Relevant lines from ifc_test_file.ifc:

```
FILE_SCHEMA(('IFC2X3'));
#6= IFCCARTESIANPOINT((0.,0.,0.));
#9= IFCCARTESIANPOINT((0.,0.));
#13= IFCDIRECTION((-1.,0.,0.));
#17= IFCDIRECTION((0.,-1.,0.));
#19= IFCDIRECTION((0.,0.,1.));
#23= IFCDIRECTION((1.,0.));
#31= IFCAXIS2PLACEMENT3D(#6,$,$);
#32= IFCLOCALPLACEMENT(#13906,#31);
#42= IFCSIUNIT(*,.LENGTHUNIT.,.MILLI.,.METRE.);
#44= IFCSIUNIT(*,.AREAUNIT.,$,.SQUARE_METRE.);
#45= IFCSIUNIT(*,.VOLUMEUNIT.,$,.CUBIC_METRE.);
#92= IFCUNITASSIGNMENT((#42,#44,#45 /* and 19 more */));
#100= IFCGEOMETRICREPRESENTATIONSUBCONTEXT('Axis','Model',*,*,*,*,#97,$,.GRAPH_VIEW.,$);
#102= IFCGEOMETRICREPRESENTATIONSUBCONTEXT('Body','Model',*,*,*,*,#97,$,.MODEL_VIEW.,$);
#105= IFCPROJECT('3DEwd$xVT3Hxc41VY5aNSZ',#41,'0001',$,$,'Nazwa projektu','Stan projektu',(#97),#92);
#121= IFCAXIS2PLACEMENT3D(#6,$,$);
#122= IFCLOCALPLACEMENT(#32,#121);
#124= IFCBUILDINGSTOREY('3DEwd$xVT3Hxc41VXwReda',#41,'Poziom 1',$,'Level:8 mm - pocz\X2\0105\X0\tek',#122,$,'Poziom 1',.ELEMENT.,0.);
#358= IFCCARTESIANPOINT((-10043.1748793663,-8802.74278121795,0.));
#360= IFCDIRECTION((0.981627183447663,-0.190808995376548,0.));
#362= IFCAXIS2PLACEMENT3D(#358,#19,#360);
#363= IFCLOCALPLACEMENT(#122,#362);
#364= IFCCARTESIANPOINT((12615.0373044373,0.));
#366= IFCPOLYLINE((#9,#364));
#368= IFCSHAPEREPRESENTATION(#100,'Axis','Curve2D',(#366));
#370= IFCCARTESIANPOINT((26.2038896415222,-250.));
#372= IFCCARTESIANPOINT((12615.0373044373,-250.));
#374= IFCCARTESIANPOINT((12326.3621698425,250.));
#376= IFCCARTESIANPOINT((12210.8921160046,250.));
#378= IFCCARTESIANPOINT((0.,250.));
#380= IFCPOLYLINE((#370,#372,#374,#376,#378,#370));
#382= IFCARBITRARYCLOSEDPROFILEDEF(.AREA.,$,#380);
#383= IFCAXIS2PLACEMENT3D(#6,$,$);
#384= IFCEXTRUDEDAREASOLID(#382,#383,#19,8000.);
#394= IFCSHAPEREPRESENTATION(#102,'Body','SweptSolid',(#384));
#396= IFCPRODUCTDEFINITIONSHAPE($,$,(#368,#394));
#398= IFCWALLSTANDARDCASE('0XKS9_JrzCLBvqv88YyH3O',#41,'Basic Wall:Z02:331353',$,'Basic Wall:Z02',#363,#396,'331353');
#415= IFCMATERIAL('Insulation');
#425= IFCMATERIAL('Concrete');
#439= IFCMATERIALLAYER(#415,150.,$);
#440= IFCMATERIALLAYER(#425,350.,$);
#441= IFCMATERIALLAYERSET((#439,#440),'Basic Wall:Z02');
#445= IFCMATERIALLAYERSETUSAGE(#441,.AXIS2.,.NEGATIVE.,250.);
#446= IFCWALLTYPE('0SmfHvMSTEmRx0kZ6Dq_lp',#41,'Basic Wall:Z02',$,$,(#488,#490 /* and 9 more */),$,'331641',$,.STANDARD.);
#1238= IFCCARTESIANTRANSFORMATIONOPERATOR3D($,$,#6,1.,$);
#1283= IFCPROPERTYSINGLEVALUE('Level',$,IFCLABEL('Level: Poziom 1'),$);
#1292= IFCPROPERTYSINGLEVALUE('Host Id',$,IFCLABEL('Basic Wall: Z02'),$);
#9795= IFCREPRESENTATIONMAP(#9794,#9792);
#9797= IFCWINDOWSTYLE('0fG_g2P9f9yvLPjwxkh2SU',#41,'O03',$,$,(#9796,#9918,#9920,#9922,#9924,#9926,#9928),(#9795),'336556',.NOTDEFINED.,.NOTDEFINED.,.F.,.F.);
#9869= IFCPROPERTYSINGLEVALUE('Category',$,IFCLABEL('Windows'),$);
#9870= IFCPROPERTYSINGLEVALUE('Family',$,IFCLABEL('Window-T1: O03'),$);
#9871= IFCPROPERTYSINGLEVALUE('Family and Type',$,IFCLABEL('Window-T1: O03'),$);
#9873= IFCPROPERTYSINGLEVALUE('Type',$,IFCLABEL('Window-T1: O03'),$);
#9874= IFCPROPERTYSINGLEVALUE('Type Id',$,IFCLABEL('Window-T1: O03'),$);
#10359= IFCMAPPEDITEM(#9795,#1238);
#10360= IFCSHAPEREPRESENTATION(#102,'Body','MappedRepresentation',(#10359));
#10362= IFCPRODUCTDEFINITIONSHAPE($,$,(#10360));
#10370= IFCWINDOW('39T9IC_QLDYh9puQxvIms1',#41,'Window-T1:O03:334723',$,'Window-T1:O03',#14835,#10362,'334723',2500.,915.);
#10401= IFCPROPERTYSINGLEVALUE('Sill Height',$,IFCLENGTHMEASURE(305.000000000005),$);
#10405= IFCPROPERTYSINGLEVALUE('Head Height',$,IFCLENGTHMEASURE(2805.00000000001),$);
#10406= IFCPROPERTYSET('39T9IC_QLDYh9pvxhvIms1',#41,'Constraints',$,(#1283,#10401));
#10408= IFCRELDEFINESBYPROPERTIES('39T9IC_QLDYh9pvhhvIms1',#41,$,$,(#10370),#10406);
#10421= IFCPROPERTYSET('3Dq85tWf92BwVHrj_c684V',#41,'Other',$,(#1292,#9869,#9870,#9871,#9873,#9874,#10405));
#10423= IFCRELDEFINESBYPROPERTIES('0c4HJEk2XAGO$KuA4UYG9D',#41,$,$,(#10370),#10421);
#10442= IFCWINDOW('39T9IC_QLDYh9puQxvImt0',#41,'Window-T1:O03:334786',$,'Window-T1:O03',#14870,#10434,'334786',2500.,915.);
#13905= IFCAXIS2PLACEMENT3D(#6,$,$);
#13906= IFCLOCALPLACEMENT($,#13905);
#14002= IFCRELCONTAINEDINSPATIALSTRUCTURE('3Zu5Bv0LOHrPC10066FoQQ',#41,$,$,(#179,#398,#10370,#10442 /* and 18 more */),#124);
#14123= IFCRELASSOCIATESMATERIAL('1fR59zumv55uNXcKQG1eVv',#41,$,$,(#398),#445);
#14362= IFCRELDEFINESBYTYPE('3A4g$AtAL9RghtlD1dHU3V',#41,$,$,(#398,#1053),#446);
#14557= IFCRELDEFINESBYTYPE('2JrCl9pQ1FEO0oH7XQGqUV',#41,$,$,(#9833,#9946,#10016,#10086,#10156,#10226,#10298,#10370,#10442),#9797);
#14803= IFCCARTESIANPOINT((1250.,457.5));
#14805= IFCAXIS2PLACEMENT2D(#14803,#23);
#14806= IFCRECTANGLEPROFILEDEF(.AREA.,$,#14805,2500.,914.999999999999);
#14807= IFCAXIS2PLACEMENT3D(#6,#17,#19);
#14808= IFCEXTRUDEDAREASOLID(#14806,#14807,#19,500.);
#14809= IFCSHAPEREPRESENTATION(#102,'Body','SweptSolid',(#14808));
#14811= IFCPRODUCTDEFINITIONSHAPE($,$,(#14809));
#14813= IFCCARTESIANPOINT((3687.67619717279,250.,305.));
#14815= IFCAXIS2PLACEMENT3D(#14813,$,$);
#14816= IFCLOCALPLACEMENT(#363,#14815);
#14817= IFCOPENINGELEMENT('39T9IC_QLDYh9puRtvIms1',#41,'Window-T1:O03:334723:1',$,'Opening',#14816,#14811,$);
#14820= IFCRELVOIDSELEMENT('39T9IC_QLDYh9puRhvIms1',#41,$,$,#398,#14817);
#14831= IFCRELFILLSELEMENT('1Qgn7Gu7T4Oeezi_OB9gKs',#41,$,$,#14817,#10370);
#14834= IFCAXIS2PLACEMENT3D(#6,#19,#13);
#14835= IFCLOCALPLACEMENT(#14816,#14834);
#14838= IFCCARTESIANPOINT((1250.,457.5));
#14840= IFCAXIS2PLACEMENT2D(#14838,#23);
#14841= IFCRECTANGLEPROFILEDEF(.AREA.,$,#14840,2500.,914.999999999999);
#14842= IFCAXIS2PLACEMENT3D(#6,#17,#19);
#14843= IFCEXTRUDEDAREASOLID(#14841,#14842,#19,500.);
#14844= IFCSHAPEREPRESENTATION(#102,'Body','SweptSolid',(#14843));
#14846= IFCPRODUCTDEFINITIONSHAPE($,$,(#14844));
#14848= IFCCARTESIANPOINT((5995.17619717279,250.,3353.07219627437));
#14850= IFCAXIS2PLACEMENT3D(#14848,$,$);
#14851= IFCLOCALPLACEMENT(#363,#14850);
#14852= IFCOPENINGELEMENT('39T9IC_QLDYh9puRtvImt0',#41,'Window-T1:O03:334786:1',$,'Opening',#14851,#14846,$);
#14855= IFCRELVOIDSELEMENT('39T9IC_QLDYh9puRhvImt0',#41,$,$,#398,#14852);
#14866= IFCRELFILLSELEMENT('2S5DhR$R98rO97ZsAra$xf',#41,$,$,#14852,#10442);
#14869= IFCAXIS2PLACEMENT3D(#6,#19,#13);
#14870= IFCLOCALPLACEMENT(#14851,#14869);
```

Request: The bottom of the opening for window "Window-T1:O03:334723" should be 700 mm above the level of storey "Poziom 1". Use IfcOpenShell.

```python
import numpy as np
import ifcopenshell
import ifcopenshell.api.geometry
import ifcopenshell.api.pset
import ifcopenshell.geom
import ifcopenshell.util.element
import ifcopenshell.util.placement
import ifcopenshell.util.shape
import ifcopenshell.util.unit

model = ifcopenshell.open("ifc_test_file.ifc")
unit_scale = ifcopenshell.util.unit.calculate_unit_scale(model)

window = model.by_guid("39T9IC_QLDYh9puQxvIms1")
opening = window.FillsVoids[0].RelatingOpeningElement
storey = ifcopenshell.util.element.get_container(window, ifc_class="IfcBuildingStorey")
level = ifcopenshell.util.placement.get_local_placement(storey.ObjectPlacement)[2, 3]

# The opening's origin need not be at the sill, so measure its lowest point.
shape = ifcopenshell.geom.create_shape(ifcopenshell.geom.settings(), opening)
bottom = ifcopenshell.util.shape.get_shape_bottom_elevation(shape, shape.geometry) / unit_scale
dz = level + 0.7 / unit_scale - bottom

shift = np.array([0.0, 0.0, dz])
# The window is placed relative to its opening, so it follows when the opening moves.
matrix = ifcopenshell.util.placement.get_local_placement(opening.ObjectPlacement)
matrix[:3, 3] += shift
ifcopenshell.api.geometry.edit_object_placement(
    model, product=opening, matrix=matrix, is_si=False, should_transform_children=True
)

# Keep the stored heights in step.
pset = model.by_id(ifcopenshell.util.element.get_pset(window, "Constraints", should_inherit=False)["id"])
ifcopenshell.api.pset.edit_pset(model, pset=pset, properties={
    "Sill Height": model.create_entity("IfcLengthMeasure", ifcopenshell.util.element.get_pset(window, "Constraints", "Sill Height") + dz),
})
pset = model.by_id(ifcopenshell.util.element.get_pset(window, "Other", should_inherit=False)["id"])
ifcopenshell.api.pset.edit_pset(model, pset=pset, properties={
    "Head Height": model.create_entity("IfcLengthMeasure", ifcopenshell.util.element.get_pset(window, "Other", "Head Height") + dz),
})

print(f"moved by {dz * unit_scale:+.3f} m")

model.write("ifc_test_file_updated.ifc")
```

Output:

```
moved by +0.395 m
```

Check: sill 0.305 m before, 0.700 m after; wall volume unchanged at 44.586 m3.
